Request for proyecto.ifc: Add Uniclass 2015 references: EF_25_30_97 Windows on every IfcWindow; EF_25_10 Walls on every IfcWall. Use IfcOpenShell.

First a look at what the model holds.

```python
import ifcopenshell

model = ifcopenshell.open("proyecto.ifc")
print(model.schema)
print("classifications:", [c.Name for c in model.by_type("IfcClassification")])
for ifc_class in ("IfcDoor", "IfcRoof", "IfcStair", "IfcWall", "IfcWindow"):
    print(ifc_class, len(model.by_type(ifc_class)))
```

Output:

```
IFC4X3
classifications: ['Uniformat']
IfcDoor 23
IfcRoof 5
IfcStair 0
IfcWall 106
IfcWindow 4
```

```python
import ifcopenshell
import ifcopenshell.api.classification

model = ifcopenshell.open("proyecto.ifc")

system = ifcopenshell.api.classification.add_classification(model, classification="Uniclass 2015")

codes = {
    "IfcWindow": ("EF_25_30_97", "Windows"),
    "IfcWall": ("EF_25_10", "Walls"),
}
for ifc_class, (code, name) in codes.items():
    products = model.by_type(ifc_class)
    ifcopenshell.api.classification.add_reference(
        model, products=products, classification=system, identification=code, name=name
    )
    print(code, len(products))

model.write("proyecto_updated.ifc")
```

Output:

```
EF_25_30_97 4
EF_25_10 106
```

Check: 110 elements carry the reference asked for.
